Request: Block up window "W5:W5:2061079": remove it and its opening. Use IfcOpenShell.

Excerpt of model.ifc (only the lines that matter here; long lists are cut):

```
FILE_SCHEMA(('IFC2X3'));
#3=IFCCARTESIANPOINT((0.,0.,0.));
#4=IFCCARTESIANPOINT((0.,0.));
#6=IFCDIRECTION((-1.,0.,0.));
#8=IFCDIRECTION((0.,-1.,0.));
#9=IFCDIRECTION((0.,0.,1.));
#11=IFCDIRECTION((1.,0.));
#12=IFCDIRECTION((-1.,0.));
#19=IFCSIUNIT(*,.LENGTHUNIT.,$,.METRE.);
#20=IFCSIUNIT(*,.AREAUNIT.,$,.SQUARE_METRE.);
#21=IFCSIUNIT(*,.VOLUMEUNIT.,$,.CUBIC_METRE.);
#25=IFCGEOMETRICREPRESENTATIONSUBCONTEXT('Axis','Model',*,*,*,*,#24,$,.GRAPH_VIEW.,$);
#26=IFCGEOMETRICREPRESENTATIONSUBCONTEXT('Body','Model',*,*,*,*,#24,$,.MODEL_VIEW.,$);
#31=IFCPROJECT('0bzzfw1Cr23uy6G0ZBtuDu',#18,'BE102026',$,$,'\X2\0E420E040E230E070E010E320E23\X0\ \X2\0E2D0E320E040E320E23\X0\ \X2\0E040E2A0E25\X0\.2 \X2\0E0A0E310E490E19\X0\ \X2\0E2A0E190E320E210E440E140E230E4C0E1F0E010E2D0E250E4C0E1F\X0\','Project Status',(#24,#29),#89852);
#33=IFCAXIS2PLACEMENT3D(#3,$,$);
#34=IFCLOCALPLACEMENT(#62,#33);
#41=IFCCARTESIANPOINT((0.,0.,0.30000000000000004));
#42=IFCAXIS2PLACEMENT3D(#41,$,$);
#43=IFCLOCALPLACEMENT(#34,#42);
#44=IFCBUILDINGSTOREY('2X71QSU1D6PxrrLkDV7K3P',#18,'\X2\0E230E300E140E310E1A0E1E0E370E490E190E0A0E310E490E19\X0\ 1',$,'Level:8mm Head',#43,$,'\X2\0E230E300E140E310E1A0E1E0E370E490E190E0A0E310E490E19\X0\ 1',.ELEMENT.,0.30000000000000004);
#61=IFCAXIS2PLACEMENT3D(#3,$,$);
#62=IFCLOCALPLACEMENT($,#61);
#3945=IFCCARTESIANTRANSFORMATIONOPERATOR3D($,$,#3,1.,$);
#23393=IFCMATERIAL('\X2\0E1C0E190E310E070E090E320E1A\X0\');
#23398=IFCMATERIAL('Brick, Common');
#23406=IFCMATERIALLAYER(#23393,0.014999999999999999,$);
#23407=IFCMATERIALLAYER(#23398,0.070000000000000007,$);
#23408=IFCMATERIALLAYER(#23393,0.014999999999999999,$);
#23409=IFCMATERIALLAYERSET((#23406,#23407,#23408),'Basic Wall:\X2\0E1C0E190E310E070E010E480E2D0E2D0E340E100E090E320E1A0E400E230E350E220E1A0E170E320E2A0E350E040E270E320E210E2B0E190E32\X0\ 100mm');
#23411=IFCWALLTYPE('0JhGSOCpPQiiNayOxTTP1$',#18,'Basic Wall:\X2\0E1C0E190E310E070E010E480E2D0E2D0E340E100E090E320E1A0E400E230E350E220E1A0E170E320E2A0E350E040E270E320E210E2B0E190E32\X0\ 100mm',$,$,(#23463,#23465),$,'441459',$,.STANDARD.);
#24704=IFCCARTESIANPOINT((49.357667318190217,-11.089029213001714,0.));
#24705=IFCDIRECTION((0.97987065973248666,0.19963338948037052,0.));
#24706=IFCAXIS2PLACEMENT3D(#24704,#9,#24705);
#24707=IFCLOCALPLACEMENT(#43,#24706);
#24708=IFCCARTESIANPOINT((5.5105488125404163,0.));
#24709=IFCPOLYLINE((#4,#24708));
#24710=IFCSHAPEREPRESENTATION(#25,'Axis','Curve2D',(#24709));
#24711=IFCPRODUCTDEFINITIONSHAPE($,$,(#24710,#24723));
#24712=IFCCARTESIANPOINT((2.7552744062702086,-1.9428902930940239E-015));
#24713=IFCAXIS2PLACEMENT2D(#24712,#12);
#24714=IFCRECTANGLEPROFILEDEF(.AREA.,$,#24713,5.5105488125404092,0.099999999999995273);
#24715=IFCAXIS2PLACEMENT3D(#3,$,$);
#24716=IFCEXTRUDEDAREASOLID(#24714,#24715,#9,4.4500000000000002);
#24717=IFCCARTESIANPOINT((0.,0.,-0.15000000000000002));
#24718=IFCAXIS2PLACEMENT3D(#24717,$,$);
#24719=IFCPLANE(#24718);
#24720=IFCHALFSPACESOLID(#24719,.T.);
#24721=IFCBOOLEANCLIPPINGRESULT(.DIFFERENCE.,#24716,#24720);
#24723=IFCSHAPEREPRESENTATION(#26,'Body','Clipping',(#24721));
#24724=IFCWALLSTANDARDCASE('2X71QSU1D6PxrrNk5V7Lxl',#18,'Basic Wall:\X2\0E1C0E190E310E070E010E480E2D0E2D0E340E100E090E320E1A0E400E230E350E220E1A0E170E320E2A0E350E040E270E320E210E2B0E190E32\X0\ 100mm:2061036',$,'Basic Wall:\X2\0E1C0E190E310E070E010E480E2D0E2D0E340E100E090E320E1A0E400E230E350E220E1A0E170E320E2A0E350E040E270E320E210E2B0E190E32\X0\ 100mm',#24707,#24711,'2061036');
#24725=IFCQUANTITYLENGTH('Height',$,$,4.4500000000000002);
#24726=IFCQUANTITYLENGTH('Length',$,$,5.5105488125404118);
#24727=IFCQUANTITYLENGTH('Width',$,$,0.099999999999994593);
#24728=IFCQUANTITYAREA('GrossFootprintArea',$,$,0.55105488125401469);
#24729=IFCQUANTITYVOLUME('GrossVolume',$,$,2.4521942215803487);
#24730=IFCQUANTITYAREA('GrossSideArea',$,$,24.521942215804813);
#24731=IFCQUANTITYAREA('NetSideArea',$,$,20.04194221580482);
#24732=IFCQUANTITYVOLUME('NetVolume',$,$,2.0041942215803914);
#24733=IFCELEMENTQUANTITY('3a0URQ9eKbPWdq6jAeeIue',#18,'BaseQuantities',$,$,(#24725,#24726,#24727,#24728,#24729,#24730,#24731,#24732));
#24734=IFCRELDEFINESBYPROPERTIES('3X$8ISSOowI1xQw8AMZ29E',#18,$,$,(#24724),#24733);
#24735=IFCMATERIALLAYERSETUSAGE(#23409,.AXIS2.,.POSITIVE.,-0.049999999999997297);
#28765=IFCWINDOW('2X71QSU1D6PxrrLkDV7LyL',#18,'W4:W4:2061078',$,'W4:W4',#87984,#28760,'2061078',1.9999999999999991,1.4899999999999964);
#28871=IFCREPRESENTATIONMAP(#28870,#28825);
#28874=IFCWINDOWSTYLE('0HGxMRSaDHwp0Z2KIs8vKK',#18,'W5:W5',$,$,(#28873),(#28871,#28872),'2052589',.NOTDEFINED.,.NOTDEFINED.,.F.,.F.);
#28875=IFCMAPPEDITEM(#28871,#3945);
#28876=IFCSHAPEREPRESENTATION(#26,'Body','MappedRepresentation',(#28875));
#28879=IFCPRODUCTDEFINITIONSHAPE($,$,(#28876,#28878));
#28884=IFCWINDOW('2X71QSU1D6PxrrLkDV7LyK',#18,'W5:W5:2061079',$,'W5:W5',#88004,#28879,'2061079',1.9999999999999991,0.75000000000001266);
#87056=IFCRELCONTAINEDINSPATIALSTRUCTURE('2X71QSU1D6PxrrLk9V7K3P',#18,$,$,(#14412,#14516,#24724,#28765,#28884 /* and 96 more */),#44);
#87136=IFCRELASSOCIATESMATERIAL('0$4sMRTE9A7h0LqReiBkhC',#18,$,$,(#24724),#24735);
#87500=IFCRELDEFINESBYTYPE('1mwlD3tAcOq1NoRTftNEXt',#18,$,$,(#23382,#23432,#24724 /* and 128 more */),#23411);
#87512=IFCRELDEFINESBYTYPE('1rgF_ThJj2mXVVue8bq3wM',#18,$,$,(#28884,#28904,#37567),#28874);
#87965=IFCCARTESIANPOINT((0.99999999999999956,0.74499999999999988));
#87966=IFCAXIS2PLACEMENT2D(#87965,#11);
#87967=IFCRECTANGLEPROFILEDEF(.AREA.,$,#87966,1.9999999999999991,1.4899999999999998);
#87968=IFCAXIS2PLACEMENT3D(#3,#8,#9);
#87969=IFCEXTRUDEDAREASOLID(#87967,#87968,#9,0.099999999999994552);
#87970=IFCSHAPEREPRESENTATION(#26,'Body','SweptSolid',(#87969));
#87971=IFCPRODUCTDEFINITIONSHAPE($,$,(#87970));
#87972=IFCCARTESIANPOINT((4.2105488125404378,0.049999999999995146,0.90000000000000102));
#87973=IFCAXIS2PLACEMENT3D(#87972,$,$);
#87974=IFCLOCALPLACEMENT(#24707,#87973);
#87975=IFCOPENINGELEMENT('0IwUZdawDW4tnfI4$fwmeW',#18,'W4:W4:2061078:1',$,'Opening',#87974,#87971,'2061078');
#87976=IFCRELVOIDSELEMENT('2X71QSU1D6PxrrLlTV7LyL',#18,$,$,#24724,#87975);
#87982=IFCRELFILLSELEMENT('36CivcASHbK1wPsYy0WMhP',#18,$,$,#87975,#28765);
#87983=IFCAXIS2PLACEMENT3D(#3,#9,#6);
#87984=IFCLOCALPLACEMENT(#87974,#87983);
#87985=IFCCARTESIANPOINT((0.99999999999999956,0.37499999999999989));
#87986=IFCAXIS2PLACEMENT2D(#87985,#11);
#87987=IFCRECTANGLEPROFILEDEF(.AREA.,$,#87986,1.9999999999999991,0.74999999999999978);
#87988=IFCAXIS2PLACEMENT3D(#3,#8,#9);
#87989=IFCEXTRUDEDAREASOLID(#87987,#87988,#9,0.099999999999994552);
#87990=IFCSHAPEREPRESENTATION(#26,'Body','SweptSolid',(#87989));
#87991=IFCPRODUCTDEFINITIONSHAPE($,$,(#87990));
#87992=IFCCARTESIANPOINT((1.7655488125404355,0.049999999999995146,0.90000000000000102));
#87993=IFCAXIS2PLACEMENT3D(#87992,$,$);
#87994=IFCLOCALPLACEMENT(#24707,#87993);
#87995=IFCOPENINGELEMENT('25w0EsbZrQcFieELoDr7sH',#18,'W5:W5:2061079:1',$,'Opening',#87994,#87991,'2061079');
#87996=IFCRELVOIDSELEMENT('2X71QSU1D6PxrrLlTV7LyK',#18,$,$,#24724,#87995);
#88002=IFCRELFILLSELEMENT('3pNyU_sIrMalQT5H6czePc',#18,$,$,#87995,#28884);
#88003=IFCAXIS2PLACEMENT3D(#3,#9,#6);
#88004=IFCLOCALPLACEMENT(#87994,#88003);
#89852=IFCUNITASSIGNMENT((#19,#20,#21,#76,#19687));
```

```python
import ifcopenshell
import ifcopenshell.api.feature
import ifcopenshell.api.pset
import ifcopenshell.api.root
import ifcopenshell.geom
import ifcopenshell.util.element
import ifcopenshell.util.shape
import ifcopenshell.util.unit

model = ifcopenshell.open("model.ifc")
area_scale = ifcopenshell.util.unit.calculate_unit_scale(model, "AREAUNIT")
volume_scale = ifcopenshell.util.unit.calculate_unit_scale(model, "VOLUMEUNIT")
settings = ifcopenshell.geom.settings()


def volume(element):
    """Net volume in cubic metres, openings subtracted."""
    shape = ifcopenshell.geom.create_shape(settings, element)
    return ifcopenshell.util.shape.get_volume(shape.geometry)


window = model.by_guid("2X71QSU1D6PxrrLkDV7LyK")
opening = window.FillsVoids[0].RelatingOpeningElement
wall = opening.VoidsElements[0].RelatingBuildingElement
before = volume(wall)

ifcopenshell.api.root.remove_product(model, product=window)
ifcopenshell.api.feature.remove_feature(model, feature=opening)

after = volume(wall)
thickness = 0.1  # wall thickness in metres

# Update the wall's stored quantities.
qto = model.by_id(ifcopenshell.util.element.get_pset(wall, "BaseQuantities", should_inherit=False)["id"])
ifcopenshell.api.pset.edit_qto(model, qto=qto, properties={
    "NetSideArea": after / thickness / area_scale,
    "NetVolume": after / volume_scale,
})

print(f"wall volume {before:.3f} -> {after:.3f} m3")

model.write("model_v2.ifc")
```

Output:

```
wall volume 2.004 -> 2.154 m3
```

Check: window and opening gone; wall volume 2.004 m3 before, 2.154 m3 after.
